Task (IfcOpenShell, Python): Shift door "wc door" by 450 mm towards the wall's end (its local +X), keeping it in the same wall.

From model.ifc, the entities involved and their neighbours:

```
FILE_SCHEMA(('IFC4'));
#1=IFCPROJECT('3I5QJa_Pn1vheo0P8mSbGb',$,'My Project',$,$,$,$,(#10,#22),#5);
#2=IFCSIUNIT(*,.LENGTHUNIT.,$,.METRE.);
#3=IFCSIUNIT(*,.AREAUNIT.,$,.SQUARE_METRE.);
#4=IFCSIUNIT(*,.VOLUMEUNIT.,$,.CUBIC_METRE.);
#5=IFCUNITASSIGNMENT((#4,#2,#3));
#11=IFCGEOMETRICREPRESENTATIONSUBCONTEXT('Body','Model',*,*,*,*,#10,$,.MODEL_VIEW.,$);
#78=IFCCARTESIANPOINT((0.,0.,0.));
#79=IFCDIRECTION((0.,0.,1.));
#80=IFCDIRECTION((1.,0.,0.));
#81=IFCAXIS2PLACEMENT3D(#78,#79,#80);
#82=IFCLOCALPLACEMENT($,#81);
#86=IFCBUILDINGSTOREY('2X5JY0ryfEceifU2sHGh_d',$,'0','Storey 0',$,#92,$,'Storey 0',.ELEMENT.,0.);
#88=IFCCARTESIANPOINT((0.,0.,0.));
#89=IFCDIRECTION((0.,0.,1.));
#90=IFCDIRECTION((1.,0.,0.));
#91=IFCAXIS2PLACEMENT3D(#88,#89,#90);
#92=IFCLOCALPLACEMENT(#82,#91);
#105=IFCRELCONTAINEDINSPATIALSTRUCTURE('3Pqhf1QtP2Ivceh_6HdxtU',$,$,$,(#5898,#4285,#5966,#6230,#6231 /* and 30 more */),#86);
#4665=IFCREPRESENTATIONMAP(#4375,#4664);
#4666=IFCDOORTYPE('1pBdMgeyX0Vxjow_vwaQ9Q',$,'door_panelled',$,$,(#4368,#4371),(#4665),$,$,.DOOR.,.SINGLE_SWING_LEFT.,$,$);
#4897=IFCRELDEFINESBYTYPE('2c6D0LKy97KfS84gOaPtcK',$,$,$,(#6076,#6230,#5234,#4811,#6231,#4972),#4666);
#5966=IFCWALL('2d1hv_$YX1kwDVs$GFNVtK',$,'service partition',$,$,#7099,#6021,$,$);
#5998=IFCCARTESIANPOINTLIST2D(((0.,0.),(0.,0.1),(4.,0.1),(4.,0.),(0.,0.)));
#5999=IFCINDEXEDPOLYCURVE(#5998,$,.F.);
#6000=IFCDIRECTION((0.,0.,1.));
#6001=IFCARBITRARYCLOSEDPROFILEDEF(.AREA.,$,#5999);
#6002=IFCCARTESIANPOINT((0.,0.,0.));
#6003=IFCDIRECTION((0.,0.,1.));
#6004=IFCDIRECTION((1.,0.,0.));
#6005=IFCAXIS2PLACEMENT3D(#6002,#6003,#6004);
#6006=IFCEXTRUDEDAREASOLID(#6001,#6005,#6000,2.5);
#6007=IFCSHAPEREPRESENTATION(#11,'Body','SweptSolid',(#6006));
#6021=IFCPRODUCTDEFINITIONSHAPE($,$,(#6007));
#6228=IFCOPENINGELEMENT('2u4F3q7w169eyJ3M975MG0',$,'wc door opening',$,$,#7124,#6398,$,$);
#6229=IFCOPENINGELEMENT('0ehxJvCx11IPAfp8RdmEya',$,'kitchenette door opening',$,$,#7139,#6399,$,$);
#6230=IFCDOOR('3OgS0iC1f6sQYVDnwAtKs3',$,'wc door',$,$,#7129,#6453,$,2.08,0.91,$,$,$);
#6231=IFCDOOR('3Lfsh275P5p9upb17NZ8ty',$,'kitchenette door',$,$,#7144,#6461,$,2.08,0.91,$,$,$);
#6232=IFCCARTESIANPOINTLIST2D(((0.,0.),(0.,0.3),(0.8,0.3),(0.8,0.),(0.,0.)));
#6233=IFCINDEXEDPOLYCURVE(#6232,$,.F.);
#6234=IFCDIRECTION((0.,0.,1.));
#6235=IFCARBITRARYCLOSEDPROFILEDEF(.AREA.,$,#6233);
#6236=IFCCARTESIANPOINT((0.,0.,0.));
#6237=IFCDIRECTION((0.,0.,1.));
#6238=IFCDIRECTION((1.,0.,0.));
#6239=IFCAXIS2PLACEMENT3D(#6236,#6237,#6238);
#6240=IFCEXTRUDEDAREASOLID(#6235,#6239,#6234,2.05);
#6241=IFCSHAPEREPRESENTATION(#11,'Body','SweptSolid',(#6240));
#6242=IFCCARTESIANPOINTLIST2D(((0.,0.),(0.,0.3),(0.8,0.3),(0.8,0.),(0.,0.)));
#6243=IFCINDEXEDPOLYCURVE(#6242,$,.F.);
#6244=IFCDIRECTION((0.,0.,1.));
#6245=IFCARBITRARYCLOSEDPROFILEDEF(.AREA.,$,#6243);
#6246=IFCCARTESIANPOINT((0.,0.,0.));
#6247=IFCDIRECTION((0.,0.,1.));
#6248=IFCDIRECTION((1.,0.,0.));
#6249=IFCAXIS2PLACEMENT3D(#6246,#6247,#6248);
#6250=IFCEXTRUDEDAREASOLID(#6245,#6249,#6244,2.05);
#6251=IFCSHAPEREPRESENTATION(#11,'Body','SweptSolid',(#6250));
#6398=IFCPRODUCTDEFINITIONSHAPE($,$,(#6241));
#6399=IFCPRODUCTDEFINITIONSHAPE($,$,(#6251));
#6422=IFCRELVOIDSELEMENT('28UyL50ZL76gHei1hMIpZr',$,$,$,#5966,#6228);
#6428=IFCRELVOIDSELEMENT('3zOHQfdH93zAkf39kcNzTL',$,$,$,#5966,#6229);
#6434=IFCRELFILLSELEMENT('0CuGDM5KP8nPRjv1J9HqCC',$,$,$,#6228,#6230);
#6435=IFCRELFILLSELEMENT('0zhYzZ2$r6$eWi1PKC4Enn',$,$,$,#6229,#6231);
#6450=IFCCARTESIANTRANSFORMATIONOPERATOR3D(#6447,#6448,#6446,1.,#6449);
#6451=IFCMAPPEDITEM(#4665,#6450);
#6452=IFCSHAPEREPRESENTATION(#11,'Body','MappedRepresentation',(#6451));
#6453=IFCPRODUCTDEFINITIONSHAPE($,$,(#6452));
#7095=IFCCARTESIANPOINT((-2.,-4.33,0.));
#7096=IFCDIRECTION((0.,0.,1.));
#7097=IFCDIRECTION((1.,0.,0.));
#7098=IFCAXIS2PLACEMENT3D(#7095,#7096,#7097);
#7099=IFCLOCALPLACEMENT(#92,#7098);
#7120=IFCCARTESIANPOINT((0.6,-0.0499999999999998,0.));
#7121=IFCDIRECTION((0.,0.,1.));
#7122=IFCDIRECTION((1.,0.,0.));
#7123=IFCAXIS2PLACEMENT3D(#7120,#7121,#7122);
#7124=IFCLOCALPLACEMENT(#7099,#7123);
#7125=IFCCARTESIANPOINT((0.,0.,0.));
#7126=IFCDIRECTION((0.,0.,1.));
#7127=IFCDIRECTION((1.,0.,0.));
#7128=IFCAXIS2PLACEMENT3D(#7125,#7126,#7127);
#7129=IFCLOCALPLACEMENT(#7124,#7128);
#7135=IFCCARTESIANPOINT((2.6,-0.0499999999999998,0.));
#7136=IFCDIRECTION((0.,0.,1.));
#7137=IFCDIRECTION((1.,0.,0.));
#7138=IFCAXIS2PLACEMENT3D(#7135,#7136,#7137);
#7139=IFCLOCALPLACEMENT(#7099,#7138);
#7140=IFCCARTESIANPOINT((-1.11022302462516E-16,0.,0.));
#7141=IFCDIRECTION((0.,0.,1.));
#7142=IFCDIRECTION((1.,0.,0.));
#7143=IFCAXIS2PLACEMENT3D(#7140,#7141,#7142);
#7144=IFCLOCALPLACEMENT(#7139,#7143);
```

```python
import ifcopenshell
import ifcopenshell.api.geometry
import ifcopenshell.util.placement
import ifcopenshell.util.unit

model = ifcopenshell.open("model.ifc")
unit_scale = ifcopenshell.util.unit.calculate_unit_scale(model)

door = model.by_id(6230)
opening = door.FillsVoids[0].RelatingOpeningElement
wall = opening.VoidsElements[0].RelatingBuildingElement

wall_matrix = ifcopenshell.util.placement.get_local_placement(wall.ObjectPlacement)
shift = wall_matrix[:3, 0] * 0.45 / unit_scale
before = ifcopenshell.util.placement.get_local_placement(door.ObjectPlacement)[:3, 3].copy()

# The door is placed relative to its opening, so it follows when the opening moves.
matrix = ifcopenshell.util.placement.get_local_placement(opening.ObjectPlacement)
matrix[:3, 3] += shift
ifcopenshell.api.geometry.edit_object_placement(
    model, product=opening, matrix=matrix, is_si=False, should_transform_children=True
)

after = ifcopenshell.util.placement.get_local_placement(door.ObjectPlacement)[:3, 3]
print("door moved by", (after - before).round(3) + 0.0)

model.write("model_v2.ifc")
```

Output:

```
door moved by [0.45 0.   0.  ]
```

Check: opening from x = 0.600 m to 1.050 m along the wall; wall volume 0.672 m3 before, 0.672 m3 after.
